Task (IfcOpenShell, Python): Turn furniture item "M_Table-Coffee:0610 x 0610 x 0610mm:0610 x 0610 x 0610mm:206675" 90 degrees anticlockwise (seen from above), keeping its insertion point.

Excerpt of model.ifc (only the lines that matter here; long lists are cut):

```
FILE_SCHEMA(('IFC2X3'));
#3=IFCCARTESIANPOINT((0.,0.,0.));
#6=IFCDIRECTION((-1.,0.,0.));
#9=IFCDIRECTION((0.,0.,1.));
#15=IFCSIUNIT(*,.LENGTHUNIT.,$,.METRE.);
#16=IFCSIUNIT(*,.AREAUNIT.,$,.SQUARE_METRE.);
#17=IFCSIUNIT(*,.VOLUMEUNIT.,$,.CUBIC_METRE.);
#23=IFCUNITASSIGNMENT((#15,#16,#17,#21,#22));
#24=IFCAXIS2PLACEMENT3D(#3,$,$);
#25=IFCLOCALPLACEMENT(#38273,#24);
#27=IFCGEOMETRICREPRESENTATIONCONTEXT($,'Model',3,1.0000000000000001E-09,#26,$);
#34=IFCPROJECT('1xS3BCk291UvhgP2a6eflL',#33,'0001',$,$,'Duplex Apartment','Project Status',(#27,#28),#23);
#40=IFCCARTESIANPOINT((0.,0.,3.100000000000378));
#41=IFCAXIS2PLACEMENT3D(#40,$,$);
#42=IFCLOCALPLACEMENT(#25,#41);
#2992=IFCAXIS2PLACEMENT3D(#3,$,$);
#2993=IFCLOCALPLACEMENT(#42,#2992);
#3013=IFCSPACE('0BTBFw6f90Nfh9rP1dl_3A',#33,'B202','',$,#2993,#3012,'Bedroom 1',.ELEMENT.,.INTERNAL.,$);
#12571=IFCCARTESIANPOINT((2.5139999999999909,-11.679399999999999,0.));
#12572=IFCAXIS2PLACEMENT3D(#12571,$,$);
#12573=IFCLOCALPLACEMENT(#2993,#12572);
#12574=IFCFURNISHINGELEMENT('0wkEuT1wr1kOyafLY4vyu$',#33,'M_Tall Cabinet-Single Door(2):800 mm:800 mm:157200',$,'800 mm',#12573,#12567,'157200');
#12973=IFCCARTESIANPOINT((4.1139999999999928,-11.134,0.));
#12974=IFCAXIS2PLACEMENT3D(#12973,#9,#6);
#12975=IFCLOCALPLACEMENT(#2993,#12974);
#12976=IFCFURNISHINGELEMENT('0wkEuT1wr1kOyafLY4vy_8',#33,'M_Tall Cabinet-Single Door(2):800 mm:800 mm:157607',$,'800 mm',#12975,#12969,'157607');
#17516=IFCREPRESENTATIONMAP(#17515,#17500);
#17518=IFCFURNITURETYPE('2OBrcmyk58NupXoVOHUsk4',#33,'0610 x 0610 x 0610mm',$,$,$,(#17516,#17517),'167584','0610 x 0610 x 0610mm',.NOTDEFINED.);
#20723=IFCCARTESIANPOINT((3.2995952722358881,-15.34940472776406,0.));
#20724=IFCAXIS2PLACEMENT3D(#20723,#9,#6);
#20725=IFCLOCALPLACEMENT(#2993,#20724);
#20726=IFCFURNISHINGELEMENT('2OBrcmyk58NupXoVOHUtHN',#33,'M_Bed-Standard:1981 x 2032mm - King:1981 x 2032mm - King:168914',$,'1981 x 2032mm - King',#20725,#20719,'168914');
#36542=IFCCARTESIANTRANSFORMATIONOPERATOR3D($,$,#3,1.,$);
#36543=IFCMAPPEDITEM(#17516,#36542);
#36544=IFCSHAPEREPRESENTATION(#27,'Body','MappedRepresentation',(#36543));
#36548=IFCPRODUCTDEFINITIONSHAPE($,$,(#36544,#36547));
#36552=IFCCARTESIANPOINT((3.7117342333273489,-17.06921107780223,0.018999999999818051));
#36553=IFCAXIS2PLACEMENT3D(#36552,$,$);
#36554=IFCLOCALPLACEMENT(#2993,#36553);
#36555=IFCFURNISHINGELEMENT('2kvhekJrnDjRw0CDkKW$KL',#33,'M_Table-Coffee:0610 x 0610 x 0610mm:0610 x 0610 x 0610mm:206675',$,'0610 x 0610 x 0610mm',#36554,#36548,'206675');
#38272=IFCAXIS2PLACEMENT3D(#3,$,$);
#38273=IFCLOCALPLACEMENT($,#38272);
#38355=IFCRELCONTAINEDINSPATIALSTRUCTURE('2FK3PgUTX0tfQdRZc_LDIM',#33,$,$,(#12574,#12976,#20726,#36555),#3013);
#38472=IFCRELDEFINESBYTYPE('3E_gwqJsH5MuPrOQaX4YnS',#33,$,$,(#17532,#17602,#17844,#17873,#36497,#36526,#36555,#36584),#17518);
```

```python
import ifcopenshell
import ifcopenshell.api.geometry
import ifcopenshell.util.placement

model = ifcopenshell.open("model.ifc")

item = model.by_id(36555)
matrix = ifcopenshell.util.placement.get_local_placement(item.ObjectPlacement)
matrix = matrix @ ifcopenshell.util.placement.rotation(90, "Z")
ifcopenshell.api.geometry.edit_object_placement(model, product=item, matrix=matrix, is_si=False)

print(ifcopenshell.util.placement.get_local_placement(item.ObjectPlacement).round(3) + 0.0)

model.write("model_updated.ifc")
```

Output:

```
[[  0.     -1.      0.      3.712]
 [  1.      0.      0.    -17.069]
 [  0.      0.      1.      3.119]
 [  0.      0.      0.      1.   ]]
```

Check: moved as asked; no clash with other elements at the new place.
